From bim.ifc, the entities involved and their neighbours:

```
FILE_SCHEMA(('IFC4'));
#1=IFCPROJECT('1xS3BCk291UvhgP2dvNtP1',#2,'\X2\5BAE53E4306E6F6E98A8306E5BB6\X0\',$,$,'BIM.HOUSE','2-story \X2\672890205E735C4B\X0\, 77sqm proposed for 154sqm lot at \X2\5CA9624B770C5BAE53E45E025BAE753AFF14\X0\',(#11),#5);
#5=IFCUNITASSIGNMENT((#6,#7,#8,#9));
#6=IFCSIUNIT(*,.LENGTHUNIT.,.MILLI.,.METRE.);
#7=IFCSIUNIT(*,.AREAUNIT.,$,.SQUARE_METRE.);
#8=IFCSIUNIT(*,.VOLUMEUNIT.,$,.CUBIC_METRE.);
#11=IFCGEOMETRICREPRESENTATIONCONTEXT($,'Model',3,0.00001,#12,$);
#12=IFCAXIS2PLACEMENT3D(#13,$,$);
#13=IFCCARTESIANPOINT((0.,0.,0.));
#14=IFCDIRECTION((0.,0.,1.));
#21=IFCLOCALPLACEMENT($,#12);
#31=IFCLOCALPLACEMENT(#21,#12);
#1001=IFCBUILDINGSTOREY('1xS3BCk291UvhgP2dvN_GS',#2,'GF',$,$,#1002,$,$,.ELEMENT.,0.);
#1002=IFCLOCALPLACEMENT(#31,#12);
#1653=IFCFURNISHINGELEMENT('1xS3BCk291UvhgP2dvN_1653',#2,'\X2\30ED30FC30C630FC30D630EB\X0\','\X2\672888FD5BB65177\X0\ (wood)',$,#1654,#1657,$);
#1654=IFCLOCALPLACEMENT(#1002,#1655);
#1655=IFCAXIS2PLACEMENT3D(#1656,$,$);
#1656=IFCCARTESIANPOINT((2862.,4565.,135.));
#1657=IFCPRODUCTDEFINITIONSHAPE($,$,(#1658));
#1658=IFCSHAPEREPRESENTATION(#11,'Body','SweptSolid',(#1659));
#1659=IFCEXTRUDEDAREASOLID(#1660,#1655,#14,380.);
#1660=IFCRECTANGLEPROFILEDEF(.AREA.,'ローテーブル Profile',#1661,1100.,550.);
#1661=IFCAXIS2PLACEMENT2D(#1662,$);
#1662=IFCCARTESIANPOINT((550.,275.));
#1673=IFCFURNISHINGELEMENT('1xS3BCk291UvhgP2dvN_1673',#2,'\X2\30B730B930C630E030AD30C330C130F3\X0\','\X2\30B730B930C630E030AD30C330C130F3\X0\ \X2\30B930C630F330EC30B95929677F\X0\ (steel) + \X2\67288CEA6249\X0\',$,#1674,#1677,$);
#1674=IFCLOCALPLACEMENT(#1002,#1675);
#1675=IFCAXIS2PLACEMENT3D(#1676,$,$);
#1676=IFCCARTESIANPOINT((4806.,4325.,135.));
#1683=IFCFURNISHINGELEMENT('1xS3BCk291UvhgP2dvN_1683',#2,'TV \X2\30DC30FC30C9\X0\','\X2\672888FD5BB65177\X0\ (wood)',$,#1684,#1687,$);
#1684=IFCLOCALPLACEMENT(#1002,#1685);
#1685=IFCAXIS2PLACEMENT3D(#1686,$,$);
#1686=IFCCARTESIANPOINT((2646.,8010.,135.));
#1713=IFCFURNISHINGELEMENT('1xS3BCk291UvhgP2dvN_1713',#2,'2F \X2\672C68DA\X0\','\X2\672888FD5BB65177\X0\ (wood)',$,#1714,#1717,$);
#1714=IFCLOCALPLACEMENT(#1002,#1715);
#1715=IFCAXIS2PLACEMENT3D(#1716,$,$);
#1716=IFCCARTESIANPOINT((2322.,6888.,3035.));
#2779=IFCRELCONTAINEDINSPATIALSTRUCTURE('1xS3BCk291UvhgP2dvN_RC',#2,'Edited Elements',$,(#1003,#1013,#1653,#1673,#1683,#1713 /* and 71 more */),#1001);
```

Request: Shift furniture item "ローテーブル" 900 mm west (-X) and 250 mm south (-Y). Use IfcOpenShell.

```python
import ifcopenshell
import ifcopenshell.api.geometry
import ifcopenshell.util.placement

model = ifcopenshell.open("bim.ifc")

item = model.by_guid("1xS3BCk291UvhgP2dvN_1653")
matrix = ifcopenshell.util.placement.get_local_placement(item.ObjectPlacement)
matrix[0, 3] -= 900.0
matrix[1, 3] -= 250.0
ifcopenshell.api.geometry.edit_object_placement(model, product=item, matrix=matrix, is_si=False)

print(ifcopenshell.util.placement.get_local_placement(item.ObjectPlacement).round(3) + 0.0)

model.write("bim_updated.ifc")
```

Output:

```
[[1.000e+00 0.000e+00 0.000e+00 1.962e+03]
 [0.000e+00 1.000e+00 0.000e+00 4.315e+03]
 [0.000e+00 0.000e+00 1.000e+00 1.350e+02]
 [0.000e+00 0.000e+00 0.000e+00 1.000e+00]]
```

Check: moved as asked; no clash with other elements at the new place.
